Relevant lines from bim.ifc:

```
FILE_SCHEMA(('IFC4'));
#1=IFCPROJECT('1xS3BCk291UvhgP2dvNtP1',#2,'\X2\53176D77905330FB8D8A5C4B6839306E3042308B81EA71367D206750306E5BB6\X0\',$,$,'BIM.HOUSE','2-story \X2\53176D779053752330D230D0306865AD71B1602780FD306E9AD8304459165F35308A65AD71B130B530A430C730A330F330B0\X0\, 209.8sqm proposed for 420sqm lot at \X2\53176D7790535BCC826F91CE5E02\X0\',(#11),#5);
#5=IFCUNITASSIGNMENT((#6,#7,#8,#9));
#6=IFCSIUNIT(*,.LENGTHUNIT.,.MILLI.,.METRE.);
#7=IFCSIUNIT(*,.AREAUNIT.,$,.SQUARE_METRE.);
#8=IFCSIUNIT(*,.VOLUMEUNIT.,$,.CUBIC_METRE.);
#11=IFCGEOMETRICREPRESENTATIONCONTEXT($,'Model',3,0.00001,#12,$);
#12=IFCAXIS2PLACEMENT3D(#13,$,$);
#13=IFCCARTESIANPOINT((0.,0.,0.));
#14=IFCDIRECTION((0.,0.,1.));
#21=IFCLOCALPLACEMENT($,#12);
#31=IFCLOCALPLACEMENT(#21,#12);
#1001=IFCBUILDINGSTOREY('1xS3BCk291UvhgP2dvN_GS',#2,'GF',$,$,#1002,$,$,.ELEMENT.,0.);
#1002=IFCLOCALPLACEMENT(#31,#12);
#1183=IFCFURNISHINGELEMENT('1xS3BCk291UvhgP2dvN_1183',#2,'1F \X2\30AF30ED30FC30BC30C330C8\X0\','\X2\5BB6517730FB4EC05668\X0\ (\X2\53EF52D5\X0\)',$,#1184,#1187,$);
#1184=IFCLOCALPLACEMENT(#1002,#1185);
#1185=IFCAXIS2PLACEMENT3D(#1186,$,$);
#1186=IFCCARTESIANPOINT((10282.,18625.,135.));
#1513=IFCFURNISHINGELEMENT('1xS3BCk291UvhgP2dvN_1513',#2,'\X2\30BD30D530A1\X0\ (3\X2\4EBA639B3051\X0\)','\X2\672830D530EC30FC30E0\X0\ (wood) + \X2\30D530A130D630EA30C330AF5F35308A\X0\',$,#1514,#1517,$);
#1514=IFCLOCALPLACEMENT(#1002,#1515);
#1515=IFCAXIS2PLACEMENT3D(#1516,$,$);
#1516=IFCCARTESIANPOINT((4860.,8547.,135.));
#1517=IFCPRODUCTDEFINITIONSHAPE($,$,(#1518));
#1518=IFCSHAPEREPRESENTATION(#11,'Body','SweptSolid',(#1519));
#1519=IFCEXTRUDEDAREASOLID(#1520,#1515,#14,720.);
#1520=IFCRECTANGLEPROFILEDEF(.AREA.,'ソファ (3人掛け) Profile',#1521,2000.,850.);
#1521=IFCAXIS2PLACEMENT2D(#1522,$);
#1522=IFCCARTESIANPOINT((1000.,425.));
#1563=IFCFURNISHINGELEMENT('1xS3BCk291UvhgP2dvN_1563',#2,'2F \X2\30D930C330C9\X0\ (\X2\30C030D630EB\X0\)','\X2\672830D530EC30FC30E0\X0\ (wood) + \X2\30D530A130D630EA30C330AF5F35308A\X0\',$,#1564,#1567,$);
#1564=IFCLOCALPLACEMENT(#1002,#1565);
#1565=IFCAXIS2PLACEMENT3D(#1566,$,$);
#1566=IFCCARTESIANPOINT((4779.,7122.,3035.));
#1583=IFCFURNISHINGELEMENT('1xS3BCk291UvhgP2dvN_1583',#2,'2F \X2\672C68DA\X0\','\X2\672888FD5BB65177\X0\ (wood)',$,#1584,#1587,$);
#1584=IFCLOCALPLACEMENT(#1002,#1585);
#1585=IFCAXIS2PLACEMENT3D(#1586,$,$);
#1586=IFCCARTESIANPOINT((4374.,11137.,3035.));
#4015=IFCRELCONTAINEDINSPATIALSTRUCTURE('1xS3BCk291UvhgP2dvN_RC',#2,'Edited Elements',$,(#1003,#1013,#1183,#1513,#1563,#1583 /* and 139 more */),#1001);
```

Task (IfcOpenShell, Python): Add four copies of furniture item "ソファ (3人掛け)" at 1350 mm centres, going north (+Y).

```python
import numpy as np
import ifcopenshell
import ifcopenshell.api.geometry
import ifcopenshell.api.root
import ifcopenshell.util.element
import ifcopenshell.util.placement
import ifcopenshell.util.unit

model = ifcopenshell.open("bim.ifc")
unit_scale = ifcopenshell.util.unit.calculate_unit_scale(model)


def reuse_history(source, copy):
    """copy_class also copies each property set's owner history, people and application; keep the originals."""
    for rel in copy.IsDefinedBy:
        if rel.is_a("IfcRelDefinesByProperties") and (history := rel.RelatingPropertyDefinition.OwnerHistory):
            rel.RelatingPropertyDefinition.OwnerHistory = source.OwnerHistory
            ifcopenshell.util.element.remove_deep2(model, history)


source = model.by_guid("1xS3BCk291UvhgP2dvN_1513")
base = ifcopenshell.util.placement.get_local_placement(source.ObjectPlacement)
step = np.array([0.0, 1.0, 0.0]) * 1.35 / unit_scale

for i in range(1, 5):
    copy = ifcopenshell.api.root.copy_class(model, product=source)
    copy.Representation = ifcopenshell.util.element.copy_deep(
        model, source.Representation, exclude=["IfcGeometricRepresentationContext", "IfcRepresentationMap"]
    )
    reuse_history(source, copy)
    matrix = base.copy()
    matrix[:3, 3] += i * step
    print("added at", matrix[:3, 3].round(3) + 0.0)
    ifcopenshell.api.geometry.edit_object_placement(model, product=copy, matrix=matrix, is_si=False)

model.write("bim_edited.ifc")
```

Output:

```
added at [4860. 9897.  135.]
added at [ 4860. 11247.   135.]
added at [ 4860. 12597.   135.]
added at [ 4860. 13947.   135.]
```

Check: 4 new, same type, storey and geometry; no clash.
